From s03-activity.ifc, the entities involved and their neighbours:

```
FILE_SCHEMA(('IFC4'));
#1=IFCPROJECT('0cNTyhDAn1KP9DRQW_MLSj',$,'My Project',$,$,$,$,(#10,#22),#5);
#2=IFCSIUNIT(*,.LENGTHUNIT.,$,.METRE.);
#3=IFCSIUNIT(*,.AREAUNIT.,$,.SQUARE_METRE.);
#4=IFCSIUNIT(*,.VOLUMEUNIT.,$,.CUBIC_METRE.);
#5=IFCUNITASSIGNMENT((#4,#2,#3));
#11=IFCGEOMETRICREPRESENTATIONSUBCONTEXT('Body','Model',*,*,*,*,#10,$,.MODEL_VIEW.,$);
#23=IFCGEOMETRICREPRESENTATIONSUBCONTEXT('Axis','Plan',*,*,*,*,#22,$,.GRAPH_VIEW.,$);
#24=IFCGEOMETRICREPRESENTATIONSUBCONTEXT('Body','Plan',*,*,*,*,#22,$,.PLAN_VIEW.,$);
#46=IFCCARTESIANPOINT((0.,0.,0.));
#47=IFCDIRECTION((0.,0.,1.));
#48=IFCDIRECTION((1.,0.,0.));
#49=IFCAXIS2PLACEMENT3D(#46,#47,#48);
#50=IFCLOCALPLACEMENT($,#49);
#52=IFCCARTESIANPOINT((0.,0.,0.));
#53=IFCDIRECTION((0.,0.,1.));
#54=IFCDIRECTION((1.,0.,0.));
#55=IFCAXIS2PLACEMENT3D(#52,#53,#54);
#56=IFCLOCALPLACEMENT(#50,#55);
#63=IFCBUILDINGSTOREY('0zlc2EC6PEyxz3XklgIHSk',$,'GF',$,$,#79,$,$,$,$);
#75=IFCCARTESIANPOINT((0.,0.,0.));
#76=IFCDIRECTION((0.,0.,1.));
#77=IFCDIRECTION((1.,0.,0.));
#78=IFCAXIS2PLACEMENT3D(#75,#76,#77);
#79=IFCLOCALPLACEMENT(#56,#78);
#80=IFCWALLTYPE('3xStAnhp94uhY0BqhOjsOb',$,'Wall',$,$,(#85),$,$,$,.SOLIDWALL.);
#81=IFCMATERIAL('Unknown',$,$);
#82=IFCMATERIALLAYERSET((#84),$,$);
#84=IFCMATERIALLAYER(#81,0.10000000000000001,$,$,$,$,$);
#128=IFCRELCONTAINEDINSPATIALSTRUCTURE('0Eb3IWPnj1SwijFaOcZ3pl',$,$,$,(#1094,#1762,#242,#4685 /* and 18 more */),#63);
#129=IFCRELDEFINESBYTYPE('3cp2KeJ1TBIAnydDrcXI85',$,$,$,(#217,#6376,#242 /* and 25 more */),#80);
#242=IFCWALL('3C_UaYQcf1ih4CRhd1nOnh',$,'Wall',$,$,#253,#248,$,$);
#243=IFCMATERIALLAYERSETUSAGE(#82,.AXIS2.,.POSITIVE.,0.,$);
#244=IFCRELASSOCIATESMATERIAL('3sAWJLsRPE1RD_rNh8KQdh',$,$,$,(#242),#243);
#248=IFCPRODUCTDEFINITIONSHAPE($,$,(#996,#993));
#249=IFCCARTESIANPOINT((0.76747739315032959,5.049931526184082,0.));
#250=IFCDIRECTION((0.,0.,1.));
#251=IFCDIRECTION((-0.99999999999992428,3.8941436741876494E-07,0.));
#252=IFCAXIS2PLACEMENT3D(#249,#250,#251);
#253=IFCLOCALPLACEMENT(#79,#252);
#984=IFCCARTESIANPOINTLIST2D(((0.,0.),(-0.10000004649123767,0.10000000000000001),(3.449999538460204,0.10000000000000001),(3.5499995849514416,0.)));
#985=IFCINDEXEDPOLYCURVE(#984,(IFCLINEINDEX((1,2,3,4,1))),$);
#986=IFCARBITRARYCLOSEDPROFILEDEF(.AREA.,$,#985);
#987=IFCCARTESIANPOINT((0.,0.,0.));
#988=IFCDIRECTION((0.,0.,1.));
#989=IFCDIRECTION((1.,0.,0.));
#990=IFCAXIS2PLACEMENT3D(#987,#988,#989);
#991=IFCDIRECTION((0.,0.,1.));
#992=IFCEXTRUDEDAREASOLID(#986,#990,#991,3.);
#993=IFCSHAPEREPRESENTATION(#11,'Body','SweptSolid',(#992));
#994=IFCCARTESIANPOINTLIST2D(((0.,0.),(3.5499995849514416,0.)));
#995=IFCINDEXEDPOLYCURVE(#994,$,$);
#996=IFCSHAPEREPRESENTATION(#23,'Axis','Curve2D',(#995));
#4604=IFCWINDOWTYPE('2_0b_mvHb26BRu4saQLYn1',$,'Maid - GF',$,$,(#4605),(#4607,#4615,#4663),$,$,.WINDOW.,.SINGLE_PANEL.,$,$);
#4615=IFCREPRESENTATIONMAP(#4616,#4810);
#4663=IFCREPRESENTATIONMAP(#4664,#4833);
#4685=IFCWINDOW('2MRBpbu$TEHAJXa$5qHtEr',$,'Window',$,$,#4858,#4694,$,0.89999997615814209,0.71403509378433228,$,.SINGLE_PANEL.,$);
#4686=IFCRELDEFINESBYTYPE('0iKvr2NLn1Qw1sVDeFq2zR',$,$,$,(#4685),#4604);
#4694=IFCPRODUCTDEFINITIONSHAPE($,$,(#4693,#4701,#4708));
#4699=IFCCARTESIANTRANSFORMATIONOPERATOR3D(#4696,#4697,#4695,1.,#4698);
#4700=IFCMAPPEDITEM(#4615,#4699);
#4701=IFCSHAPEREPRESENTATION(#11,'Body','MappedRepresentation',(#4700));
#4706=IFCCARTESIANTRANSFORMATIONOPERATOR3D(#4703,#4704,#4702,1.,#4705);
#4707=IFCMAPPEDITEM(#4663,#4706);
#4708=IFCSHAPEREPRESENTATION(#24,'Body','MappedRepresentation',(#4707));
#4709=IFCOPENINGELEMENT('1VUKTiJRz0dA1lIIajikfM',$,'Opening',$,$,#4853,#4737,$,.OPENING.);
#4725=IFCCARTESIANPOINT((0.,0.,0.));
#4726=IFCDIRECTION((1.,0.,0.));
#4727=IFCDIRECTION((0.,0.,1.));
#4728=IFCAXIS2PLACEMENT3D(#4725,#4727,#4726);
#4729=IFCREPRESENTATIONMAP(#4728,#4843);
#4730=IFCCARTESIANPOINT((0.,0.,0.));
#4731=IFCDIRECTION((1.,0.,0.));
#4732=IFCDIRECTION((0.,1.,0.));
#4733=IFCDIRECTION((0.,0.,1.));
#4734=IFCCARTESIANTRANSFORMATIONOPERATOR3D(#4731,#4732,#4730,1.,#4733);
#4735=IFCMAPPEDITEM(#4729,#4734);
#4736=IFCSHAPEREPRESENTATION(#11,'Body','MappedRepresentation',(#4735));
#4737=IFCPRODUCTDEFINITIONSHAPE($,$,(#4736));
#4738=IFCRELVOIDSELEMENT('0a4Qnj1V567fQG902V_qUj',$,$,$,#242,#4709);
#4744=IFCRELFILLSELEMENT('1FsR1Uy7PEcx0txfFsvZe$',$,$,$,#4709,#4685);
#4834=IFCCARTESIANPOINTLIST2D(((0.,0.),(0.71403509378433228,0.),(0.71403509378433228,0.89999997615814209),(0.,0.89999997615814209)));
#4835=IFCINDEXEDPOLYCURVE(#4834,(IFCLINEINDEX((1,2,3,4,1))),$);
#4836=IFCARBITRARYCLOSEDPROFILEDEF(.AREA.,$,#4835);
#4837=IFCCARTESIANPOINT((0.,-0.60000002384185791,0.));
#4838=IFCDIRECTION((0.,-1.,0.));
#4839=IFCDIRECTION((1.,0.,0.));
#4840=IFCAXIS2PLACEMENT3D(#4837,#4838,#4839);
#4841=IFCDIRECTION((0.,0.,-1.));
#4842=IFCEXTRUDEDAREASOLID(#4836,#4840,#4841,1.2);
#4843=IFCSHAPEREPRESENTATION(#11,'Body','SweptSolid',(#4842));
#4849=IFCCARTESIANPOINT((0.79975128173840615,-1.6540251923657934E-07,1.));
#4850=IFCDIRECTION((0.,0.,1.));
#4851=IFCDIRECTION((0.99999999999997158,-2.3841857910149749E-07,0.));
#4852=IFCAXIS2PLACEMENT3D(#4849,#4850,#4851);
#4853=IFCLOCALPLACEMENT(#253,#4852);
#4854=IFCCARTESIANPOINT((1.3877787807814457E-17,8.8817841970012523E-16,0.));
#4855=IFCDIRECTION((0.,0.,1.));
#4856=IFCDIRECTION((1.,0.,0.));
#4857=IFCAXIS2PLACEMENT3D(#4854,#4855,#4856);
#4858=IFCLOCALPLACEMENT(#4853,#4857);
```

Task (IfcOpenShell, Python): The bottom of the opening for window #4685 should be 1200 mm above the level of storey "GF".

```python
import numpy as np
import ifcopenshell
import ifcopenshell.api.geometry
import ifcopenshell.geom
import ifcopenshell.util.element
import ifcopenshell.util.placement
import ifcopenshell.util.shape
import ifcopenshell.util.unit

model = ifcopenshell.open("s03-activity.ifc")
unit_scale = ifcopenshell.util.unit.calculate_unit_scale(model)

window = model.by_guid("2MRBpbu$TEHAJXa$5qHtEr")
opening = window.FillsVoids[0].RelatingOpeningElement
storey = ifcopenshell.util.element.get_container(window, ifc_class="IfcBuildingStorey")
level = ifcopenshell.util.placement.get_local_placement(storey.ObjectPlacement)[2, 3]

# The opening's origin need not be at the sill, so measure its lowest point.
shape = ifcopenshell.geom.create_shape(ifcopenshell.geom.settings(), opening)
bottom = ifcopenshell.util.shape.get_shape_bottom_elevation(shape, shape.geometry) / unit_scale
dz = level + 1.2 / unit_scale - bottom

shift = np.array([0.0, 0.0, dz])
# The window is placed relative to its opening, so it follows when the opening moves.
matrix = ifcopenshell.util.placement.get_local_placement(opening.ObjectPlacement)
matrix[:3, 3] += shift
ifcopenshell.api.geometry.edit_object_placement(
    model, product=opening, matrix=matrix, is_si=False, should_transform_children=True
)

print(f"moved by {dz * unit_scale:+.3f} m")

model.write("s03-activity_v2.ifc")
```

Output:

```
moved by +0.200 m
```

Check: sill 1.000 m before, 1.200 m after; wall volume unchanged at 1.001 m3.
